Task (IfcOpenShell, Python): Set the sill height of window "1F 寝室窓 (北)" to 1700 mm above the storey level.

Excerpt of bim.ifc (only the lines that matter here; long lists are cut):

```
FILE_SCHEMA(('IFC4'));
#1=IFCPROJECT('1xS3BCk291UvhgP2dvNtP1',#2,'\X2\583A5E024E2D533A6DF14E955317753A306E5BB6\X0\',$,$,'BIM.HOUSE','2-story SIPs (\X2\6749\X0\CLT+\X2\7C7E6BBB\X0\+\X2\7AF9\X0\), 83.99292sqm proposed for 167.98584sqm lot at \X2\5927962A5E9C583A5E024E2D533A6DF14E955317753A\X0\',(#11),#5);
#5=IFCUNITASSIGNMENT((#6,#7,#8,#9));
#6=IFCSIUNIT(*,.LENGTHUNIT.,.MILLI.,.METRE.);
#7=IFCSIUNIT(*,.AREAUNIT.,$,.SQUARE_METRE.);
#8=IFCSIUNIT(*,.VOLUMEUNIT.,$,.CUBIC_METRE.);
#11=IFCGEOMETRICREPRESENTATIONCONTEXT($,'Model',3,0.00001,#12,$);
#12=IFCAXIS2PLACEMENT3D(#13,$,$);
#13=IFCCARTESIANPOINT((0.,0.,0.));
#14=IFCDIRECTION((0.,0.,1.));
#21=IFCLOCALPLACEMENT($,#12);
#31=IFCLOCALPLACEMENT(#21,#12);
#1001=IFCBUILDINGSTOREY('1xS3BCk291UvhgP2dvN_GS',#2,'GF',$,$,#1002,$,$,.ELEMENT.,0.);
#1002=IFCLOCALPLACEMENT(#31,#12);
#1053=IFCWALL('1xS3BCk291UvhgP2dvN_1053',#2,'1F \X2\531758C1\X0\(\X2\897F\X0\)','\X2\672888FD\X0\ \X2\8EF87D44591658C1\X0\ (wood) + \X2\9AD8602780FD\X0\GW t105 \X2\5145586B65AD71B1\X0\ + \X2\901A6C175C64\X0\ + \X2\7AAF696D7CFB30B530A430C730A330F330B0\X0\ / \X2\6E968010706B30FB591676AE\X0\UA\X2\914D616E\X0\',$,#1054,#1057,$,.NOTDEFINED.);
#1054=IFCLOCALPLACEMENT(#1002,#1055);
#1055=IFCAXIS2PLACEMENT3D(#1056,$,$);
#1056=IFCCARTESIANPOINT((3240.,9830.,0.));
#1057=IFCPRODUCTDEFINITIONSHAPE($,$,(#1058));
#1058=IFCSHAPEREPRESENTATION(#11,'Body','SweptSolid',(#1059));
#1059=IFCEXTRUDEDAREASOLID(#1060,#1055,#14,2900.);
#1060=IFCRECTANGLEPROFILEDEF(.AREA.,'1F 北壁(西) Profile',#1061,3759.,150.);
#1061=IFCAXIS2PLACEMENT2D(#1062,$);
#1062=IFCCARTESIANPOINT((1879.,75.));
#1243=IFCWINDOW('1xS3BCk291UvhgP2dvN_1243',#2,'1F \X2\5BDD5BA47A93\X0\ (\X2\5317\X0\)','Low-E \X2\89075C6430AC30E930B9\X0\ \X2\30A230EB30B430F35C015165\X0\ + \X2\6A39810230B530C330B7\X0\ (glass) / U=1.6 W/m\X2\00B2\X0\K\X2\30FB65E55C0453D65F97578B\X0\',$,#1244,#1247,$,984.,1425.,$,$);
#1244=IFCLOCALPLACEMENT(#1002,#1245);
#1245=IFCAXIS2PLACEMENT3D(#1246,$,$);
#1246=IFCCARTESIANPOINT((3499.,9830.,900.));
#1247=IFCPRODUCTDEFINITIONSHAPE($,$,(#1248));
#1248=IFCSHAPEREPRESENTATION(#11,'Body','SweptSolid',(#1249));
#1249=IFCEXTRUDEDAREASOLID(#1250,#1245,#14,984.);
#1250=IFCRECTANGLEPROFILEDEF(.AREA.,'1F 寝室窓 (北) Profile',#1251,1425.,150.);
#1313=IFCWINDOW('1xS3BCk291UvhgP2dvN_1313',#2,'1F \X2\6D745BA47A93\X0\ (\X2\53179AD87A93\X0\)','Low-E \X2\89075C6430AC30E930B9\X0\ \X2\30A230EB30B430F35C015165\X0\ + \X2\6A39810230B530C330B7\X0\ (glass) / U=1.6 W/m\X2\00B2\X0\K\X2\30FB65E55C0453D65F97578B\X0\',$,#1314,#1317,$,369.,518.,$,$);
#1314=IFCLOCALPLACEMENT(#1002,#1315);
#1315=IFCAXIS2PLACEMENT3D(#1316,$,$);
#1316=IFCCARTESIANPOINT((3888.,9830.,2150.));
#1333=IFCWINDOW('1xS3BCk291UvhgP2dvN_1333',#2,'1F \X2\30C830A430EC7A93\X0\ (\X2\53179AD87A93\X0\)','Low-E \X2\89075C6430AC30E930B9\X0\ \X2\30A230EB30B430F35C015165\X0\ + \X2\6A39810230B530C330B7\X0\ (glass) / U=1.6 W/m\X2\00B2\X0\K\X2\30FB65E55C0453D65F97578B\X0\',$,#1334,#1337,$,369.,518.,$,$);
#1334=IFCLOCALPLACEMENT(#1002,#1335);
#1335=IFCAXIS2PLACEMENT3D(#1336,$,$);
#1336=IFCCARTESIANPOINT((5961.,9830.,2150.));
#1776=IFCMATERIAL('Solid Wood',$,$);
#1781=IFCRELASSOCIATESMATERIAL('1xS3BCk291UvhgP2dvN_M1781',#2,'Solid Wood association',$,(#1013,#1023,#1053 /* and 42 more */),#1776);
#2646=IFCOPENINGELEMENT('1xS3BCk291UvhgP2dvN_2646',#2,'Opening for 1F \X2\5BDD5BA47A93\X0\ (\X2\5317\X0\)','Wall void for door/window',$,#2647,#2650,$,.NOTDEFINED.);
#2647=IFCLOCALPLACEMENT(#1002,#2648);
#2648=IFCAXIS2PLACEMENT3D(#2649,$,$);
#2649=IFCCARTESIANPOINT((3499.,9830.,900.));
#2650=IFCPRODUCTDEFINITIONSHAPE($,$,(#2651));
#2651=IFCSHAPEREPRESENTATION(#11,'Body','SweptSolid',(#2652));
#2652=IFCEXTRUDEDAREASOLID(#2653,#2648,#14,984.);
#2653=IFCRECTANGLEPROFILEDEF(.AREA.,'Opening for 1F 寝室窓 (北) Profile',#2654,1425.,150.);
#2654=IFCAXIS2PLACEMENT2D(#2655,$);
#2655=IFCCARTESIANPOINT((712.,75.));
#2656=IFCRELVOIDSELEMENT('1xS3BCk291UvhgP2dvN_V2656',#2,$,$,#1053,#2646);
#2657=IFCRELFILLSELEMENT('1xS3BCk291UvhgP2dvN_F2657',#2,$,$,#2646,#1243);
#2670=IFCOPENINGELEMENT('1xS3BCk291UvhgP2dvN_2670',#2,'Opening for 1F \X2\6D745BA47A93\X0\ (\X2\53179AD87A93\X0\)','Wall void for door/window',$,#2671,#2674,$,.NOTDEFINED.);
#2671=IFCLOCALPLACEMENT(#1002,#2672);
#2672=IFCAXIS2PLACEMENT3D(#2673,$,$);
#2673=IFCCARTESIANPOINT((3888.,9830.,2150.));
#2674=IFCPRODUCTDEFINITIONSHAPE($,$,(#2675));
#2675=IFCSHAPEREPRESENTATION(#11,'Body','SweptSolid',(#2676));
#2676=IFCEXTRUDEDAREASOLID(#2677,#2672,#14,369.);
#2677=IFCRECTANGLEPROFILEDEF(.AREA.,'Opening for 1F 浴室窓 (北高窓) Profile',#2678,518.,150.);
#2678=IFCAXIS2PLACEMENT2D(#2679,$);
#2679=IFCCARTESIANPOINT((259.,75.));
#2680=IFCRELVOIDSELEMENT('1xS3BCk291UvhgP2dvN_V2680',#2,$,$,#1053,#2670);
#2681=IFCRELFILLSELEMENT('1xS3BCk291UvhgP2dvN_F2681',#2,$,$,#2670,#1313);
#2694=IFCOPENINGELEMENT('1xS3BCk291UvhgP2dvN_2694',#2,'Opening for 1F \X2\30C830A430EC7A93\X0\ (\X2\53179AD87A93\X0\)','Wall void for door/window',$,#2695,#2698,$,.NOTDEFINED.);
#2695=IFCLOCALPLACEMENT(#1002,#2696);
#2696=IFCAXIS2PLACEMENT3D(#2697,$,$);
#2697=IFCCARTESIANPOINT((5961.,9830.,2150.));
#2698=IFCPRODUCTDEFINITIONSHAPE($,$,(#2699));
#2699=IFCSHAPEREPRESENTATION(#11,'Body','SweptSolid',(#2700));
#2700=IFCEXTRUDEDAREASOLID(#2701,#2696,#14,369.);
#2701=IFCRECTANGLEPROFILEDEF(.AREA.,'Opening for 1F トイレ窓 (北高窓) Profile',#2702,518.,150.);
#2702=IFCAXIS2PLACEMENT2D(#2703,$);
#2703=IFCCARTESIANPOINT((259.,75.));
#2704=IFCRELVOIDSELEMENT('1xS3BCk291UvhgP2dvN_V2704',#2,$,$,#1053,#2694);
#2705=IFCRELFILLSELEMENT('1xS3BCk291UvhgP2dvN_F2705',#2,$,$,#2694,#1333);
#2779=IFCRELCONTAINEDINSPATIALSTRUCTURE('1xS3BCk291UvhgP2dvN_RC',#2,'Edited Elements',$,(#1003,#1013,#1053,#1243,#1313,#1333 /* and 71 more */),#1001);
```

```python
import numpy as np
import ifcopenshell
import ifcopenshell.api.geometry
import ifcopenshell.geom
import ifcopenshell.util.element
import ifcopenshell.util.placement
import ifcopenshell.util.shape
import ifcopenshell.util.unit

model = ifcopenshell.open("bim.ifc")
unit_scale = ifcopenshell.util.unit.calculate_unit_scale(model)

window = model.by_guid("1xS3BCk291UvhgP2dvN_1243")
opening = window.FillsVoids[0].RelatingOpeningElement
storey = ifcopenshell.util.element.get_container(window, ifc_class="IfcBuildingStorey")
level = ifcopenshell.util.placement.get_local_placement(storey.ObjectPlacement)[2, 3]

# The opening's origin need not be at the sill, so measure its lowest point.
shape = ifcopenshell.geom.create_shape(ifcopenshell.geom.settings(), opening)
bottom = ifcopenshell.util.shape.get_shape_bottom_elevation(shape, shape.geometry) / unit_scale
dz = level + 1.7 / unit_scale - bottom

shift = np.array([0.0, 0.0, dz])
# The window is not placed relative to its opening, so move both.
for product in (opening, window):
    matrix = ifcopenshell.util.placement.get_local_placement(product.ObjectPlacement)
    matrix[:3, 3] += shift
    ifcopenshell.api.geometry.edit_object_placement(model, product=product, matrix=matrix, is_si=False)

print(f"moved by {dz * unit_scale:+.3f} m")

model.write("bim_v2.ifc")
```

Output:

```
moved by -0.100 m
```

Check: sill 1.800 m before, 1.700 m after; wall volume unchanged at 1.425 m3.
